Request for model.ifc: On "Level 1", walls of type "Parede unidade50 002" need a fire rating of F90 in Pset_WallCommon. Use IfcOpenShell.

First a look at what the model holds.

```python
import ifcopenshell
import ifcopenshell.util.element

model = ifcopenshell.open("model.ifc")
print(model.schema)
storey = next(s for s in model.by_type("IfcBuildingStorey") if s.Name == "Level 1")
walls = [e for e in ifcopenshell.util.element.get_decomposition(storey) if e.is_a("IfcWall")]
seen = {}
for e in walls:
    element_type = ifcopenshell.util.element.get_type(e)
    key = (element_type.Name if element_type != e and element_type else None, ifcopenshell.util.element.get_pset(e, "Pset_WallCommon", "FireRating"))
    seen[key] = seen.get(key, 0) + 1
for (name, value), count in sorted(seen.items(), key=str):
    print(count, "x", name, "|", value)
```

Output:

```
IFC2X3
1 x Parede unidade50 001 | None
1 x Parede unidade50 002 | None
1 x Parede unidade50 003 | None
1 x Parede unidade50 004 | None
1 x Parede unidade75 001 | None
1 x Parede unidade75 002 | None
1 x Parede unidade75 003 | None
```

```python
import ifcopenshell
import ifcopenshell.api.pset
import ifcopenshell.util.element

model = ifcopenshell.open("model.ifc")

storey = next(s for s in model.by_type("IfcBuildingStorey") if s.Name == "Level 1")
walls = [e for e in ifcopenshell.util.element.get_decomposition(storey) if e.is_a("IfcWall")]

count = 0
for e in walls:
    element_type = ifcopenshell.util.element.get_type(e)
    if element_type in (None, e) or element_type.Name != "Parede unidade50 002":
        continue
    # add_pset returns the element's existing set when there is one.
    pset = ifcopenshell.api.pset.add_pset(model, product=e, name="Pset_WallCommon")
    ifcopenshell.api.pset.edit_pset(model, pset=pset, properties={"FireRating": "F90"})
    count += 1

print(count, "walls updated")

model.write("model-out.ifc")
```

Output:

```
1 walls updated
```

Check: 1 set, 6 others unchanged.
